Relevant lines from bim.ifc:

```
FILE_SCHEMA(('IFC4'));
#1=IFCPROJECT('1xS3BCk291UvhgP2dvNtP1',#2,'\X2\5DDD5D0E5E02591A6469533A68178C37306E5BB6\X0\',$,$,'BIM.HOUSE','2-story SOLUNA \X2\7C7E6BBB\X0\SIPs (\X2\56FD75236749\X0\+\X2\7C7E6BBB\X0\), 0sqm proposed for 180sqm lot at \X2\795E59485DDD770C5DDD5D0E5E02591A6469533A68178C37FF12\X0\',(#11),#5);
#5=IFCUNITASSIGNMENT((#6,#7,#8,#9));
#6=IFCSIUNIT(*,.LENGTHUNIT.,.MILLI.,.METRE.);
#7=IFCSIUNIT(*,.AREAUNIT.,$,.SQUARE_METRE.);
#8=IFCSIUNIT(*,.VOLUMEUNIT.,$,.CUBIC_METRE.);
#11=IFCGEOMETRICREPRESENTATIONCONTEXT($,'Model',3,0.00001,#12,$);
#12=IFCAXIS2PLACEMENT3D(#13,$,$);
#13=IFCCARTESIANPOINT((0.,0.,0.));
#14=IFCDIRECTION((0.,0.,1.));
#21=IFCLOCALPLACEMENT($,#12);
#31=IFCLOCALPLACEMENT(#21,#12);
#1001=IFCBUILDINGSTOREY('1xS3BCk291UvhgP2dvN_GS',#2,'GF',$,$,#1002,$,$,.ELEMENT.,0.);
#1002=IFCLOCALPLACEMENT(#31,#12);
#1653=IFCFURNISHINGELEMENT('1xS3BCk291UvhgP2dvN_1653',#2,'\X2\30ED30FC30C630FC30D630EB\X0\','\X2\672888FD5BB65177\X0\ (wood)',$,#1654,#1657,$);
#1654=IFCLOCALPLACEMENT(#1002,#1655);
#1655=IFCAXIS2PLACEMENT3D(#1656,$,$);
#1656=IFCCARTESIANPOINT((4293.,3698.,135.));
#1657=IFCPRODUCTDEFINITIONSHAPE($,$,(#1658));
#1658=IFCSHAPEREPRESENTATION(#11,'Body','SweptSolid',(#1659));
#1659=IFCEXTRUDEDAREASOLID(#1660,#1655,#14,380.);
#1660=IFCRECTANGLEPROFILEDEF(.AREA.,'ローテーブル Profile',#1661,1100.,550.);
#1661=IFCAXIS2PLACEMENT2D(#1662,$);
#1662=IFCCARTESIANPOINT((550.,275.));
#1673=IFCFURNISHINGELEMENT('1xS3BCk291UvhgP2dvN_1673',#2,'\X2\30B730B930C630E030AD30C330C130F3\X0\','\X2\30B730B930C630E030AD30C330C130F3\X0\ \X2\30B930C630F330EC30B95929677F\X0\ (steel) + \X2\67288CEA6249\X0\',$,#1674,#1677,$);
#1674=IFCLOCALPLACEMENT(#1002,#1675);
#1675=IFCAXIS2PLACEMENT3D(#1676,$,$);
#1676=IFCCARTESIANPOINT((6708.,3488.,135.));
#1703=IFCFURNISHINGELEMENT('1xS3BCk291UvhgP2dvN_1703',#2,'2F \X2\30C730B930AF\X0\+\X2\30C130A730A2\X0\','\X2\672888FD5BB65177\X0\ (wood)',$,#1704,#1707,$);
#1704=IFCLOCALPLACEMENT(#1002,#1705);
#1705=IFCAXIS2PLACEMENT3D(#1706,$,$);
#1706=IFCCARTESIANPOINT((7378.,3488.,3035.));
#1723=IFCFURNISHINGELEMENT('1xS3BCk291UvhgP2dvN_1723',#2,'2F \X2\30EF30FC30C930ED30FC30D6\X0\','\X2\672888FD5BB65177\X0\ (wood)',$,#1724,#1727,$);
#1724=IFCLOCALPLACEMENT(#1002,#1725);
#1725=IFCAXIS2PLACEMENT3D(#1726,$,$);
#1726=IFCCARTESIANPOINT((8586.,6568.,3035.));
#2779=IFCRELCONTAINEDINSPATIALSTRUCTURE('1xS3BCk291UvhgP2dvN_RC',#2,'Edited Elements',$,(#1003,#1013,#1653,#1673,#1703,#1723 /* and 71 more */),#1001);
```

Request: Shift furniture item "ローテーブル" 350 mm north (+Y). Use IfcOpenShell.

```python
import ifcopenshell
import ifcopenshell.api.geometry
import ifcopenshell.util.placement
import ifcopenshell.util.unit

model = ifcopenshell.open("bim.ifc")
unit_scale = ifcopenshell.util.unit.calculate_unit_scale(model)

item = model.by_id(1653)
matrix = ifcopenshell.util.placement.get_local_placement(item.ObjectPlacement)
matrix[1, 3] += 0.35 / unit_scale
ifcopenshell.api.geometry.edit_object_placement(model, product=item, matrix=matrix, is_si=False)

print(ifcopenshell.util.placement.get_local_placement(item.ObjectPlacement).round(3) + 0.0)

model.write("bim_rev.ifc")
```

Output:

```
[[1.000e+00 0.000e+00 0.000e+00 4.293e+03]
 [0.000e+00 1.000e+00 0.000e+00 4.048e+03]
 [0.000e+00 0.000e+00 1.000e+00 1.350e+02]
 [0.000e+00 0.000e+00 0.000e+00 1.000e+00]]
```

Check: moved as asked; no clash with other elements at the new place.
